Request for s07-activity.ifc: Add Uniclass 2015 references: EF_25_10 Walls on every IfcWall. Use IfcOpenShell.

First a look at what the model holds.

```python
import ifcopenshell

model = ifcopenshell.open("s07-activity.ifc")
print(model.schema)
print("classifications:", [c.Name for c in model.by_type("IfcClassification")])
for ifc_class in ("IfcDoor", "IfcRoof", "IfcStair", "IfcWall", "IfcWindow"):
    print(ifc_class, len(model.by_type(ifc_class)))
```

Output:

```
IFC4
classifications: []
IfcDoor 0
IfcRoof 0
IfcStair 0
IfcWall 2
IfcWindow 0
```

```python
import ifcopenshell
import ifcopenshell.api.classification

model = ifcopenshell.open("s07-activity.ifc")

system = ifcopenshell.api.classification.add_classification(model, classification="Uniclass 2015")

codes = {
    "IfcWall": ("EF_25_10", "Walls"),
}
for ifc_class, (code, name) in codes.items():
    products = model.by_type(ifc_class)
    ifcopenshell.api.classification.add_reference(
        model, products=products, classification=system, identification=code, name=name
    )
    print(code, len(products))

model.write("s07-activity_updated.ifc")
```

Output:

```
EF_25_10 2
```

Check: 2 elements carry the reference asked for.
